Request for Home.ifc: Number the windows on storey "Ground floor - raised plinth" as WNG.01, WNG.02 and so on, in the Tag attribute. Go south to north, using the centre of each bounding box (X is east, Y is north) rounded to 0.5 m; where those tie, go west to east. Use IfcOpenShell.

First a look at what the model holds.

```python
import ifcopenshell
import ifcopenshell.util.element
import ifcopenshell.util.placement

model = ifcopenshell.open("Home.ifc")
print(model.schema)
storey = next(s for s in model.by_type("IfcBuildingStorey") if s.Name == "Ground floor - raised plinth")
windows = [e for e in ifcopenshell.util.element.get_decomposition(storey) if e.is_a("IfcWindow")]
for e in sorted(windows, key=lambda e: e.id()):
    origin = ifcopenshell.util.placement.get_local_placement(e.ObjectPlacement)[:3, 3]
    print(e.id(), e.Tag, e.Name, origin.round(2) + 0.0, sep=" | ")
```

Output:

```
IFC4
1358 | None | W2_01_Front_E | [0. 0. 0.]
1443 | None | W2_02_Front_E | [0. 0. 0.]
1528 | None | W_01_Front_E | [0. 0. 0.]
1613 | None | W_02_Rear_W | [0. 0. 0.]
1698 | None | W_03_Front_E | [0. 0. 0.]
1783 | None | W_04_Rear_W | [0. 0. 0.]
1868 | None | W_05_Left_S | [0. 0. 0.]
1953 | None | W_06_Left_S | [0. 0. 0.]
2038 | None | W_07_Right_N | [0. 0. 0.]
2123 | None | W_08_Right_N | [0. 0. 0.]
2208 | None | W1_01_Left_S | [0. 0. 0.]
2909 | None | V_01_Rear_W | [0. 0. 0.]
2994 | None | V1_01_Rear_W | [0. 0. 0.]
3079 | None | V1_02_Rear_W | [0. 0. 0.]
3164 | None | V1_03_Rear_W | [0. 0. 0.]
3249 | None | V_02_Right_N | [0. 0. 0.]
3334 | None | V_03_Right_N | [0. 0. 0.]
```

```python
import ifcopenshell
import ifcopenshell.geom
import ifcopenshell.util.element
import ifcopenshell.util.shape

model = ifcopenshell.open("Home.ifc")
settings = ifcopenshell.geom.settings()
settings.set("use-world-coords", True)


def centre(element):
    shape = ifcopenshell.geom.create_shape(settings, element)
    return ifcopenshell.util.shape.get_bbox_centroid(shape.geometry)


storey = next(s for s in model.by_type("IfcBuildingStorey") if s.Name == "Ground floor - raised plinth")
windows = [e for e in ifcopenshell.util.element.get_decomposition(storey) if e.is_a("IfcWindow")]

# Insertion points can sit at a corner or the storey origin, so sort by the geometry (in metres).
centres = {e: centre(e) for e in windows}
windows.sort(key=lambda e: (round(centres[e][1] / 0.5), centres[e][0]))

for i, e in enumerate(windows, start=1):
    number = f"WNG.{i:02d}"
    e.Tag = number
    print(e.id(), number)

model.write("Home_updated.ifc")
```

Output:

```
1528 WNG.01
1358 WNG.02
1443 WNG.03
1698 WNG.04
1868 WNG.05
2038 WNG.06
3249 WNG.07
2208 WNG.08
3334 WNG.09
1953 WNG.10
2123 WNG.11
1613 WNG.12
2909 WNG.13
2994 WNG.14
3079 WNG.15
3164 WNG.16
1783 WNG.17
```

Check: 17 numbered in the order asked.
